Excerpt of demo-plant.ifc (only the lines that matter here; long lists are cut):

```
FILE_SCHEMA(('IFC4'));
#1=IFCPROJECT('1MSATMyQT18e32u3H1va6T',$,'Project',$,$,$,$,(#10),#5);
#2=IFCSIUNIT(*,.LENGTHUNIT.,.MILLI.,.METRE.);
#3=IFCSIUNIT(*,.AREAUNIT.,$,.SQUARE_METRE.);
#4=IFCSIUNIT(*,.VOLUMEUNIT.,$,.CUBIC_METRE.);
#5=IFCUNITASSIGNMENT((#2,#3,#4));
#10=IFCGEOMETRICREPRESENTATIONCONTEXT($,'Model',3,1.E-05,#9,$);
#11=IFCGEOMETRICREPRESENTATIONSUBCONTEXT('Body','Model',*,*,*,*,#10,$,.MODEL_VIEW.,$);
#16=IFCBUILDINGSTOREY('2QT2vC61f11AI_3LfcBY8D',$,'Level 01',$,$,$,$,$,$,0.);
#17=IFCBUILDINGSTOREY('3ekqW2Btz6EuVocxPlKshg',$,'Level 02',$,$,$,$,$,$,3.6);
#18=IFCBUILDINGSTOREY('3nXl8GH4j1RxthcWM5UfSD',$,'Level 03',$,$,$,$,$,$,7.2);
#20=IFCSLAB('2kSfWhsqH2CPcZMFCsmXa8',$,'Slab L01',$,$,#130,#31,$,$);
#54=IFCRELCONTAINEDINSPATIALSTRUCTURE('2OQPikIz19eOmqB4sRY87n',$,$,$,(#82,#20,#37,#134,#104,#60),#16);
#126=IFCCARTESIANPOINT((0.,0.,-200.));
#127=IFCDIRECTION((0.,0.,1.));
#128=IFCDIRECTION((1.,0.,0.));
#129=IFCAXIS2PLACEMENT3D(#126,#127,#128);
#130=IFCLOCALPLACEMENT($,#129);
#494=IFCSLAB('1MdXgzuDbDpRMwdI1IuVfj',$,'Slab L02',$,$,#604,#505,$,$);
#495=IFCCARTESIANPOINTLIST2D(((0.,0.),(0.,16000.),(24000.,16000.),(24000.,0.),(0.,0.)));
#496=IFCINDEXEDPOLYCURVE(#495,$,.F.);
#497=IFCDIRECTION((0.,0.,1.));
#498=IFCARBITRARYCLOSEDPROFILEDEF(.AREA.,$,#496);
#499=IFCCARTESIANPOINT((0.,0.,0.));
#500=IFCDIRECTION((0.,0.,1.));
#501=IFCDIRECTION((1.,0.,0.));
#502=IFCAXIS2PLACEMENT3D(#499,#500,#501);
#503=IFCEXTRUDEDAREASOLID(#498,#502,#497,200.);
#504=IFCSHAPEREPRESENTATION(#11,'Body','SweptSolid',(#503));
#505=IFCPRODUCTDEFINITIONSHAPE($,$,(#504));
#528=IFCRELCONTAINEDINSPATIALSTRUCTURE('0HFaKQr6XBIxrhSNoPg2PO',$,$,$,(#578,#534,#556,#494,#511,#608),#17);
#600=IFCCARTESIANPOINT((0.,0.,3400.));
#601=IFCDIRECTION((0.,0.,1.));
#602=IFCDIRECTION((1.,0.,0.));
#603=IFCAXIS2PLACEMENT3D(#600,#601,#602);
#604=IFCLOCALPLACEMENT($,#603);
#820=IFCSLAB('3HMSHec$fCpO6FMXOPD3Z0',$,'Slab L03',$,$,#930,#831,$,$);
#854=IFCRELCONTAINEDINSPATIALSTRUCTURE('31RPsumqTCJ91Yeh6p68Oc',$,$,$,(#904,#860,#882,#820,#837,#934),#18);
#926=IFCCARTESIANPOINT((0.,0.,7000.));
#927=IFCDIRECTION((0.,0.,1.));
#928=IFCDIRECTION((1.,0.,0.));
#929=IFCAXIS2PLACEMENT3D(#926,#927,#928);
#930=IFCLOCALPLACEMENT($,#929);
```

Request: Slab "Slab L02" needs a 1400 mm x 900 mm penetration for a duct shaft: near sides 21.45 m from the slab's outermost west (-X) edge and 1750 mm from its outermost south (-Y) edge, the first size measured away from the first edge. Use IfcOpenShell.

```python
import numpy as np
import ifcopenshell
import ifcopenshell.api.feature
import ifcopenshell.api.geometry
import ifcopenshell.api.root
import ifcopenshell.geom
import ifcopenshell.util.placement
import ifcopenshell.util.representation
import ifcopenshell.util.shape
import ifcopenshell.util.unit

model = ifcopenshell.open("demo-plant.ifc")
unit_scale = ifcopenshell.util.unit.calculate_unit_scale(model)
settings = ifcopenshell.geom.settings()


def volume(element):
    """Net volume in cubic metres, openings subtracted."""
    shape = ifcopenshell.geom.create_shape(settings, element)
    return ifcopenshell.util.shape.get_volume(shape.geometry)


slab = model.by_id(494)
before = volume(slab)

# Extent in the slab's own axes, in metres. The edges named are its -X and -Y sides.
slab_shape = ifcopenshell.geom.create_shape(settings, slab)
vertices = ifcopenshell.util.shape.get_vertices(slab_shape.geometry)
x_min, y_min, bottom = vertices.min(axis=0)
top = vertices[:, 2].max()

opening = ifcopenshell.api.root.create_entity(model, ifc_class="IfcOpeningElement", name="Duct shaft opening", predefined_type="OPENING")
context = ifcopenshell.util.representation.get_context(model, "Model", "Body", "MODEL_VIEW")
width, depth = 1.4, 0.9
outline = [(0.0, 0.0), (width, 0.0), (width, depth), (0.0, depth), (0.0, 0.0)]
# Overshoot both faces by 50 mm so the cut is clean.
shape = ifcopenshell.api.geometry.add_slab_representation(
    model, context=context, depth=top - bottom + 0.1, polyline=outline
)
ifcopenshell.api.geometry.assign_representation(model, product=opening, representation=shape)

matrix = ifcopenshell.util.placement.get_local_placement(slab.ObjectPlacement)
matrix[:, 3] = matrix @ np.append(np.array([x_min + 21.45, y_min + 1.75, bottom - 0.05]) / unit_scale, 1.0)
ifcopenshell.api.geometry.edit_object_placement(model, product=opening, matrix=matrix, is_si=False)
ifcopenshell.api.feature.add_feature(model, feature=opening, element=slab)

after = volume(slab)

print(f"slab volume {before:.3f} -> {after:.3f} m3")

model.write("demo-plant_edited.ifc")
```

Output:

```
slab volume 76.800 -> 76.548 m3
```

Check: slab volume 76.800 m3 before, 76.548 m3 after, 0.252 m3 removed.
